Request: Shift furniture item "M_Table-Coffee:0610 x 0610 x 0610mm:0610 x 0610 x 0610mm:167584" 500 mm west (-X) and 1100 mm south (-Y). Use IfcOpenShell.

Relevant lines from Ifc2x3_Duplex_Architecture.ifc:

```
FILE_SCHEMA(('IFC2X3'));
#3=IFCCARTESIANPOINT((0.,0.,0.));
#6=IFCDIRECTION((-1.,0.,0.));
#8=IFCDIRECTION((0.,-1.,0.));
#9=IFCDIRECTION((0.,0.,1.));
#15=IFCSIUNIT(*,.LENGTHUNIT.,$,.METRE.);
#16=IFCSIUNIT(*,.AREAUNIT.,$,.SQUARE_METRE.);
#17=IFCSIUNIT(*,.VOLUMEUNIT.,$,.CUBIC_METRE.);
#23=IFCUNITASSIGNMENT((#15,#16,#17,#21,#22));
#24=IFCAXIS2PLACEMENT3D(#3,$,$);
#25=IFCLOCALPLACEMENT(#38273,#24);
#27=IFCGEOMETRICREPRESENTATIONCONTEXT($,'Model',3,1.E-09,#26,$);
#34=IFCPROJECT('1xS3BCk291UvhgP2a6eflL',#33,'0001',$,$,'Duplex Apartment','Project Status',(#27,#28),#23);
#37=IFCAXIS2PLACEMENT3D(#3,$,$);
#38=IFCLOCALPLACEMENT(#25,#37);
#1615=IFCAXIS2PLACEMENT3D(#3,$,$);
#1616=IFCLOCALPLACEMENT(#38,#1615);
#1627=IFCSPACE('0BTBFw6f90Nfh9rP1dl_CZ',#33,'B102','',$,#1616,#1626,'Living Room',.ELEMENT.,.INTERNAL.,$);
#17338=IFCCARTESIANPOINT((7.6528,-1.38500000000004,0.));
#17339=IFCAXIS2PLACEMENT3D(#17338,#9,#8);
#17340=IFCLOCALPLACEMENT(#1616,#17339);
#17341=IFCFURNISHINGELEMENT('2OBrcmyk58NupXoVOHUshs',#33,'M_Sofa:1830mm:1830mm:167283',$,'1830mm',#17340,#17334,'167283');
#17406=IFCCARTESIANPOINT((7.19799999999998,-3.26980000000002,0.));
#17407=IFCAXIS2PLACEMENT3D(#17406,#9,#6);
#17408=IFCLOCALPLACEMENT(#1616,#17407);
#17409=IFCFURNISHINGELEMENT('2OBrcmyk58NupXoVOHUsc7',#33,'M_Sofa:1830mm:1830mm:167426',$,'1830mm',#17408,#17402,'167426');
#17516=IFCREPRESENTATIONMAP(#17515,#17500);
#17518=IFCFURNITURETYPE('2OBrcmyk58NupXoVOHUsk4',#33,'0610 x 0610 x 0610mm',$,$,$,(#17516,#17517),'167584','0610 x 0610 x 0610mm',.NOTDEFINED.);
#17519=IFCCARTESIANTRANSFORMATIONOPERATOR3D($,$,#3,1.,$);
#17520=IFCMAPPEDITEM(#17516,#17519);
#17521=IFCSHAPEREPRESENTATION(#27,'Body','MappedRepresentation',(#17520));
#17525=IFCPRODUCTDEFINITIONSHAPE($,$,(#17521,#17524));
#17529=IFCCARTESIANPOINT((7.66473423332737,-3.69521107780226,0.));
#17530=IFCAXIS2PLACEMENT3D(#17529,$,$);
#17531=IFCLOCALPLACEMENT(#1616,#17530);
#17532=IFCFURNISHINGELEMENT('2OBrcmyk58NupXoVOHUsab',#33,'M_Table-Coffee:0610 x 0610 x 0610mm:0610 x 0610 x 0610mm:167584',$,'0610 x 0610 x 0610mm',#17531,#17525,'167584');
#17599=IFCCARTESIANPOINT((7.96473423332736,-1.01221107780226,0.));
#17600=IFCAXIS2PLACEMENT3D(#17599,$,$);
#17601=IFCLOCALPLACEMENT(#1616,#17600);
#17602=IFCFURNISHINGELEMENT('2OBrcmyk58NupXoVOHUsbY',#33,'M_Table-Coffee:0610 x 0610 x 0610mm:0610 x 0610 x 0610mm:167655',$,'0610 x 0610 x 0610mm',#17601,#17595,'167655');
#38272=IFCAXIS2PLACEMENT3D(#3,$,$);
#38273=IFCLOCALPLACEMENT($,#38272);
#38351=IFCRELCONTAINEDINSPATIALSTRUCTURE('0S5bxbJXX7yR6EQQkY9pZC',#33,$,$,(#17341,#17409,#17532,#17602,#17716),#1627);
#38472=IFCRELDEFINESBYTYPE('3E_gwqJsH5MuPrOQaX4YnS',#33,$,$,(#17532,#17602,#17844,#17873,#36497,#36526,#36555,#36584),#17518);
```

```python
import ifcopenshell
import ifcopenshell.api.geometry
import ifcopenshell.util.placement
import ifcopenshell.util.unit

model = ifcopenshell.open("Ifc2x3_Duplex_Architecture.ifc")
unit_scale = ifcopenshell.util.unit.calculate_unit_scale(model)

item = model.by_id(17532)
matrix = ifcopenshell.util.placement.get_local_placement(item.ObjectPlacement)
matrix[0, 3] -= 0.5 / unit_scale
matrix[1, 3] -= 1.1 / unit_scale
ifcopenshell.api.geometry.edit_object_placement(model, product=item, matrix=matrix, is_si=False)

print(ifcopenshell.util.placement.get_local_placement(item.ObjectPlacement).round(3) + 0.0)

model.write("Ifc2x3_Duplex_Architecture_rev.ifc")
```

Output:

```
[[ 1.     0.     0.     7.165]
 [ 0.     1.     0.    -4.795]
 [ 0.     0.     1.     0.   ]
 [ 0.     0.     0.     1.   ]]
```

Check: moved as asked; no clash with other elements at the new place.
